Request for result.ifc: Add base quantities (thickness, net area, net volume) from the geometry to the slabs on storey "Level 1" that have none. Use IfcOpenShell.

First a look at what the model holds.

```python
import ifcopenshell
import ifcopenshell.util.element
import ifcopenshell.util.unit

model = ifcopenshell.open("result.ifc")
print(model.schema)
for unit_type in ("LENGTHUNIT", "AREAUNIT", "VOLUMEUNIT"):
    print(unit_type, ifcopenshell.util.unit.calculate_unit_scale(model, unit_type))
storey = next(s for s in model.by_type("IfcBuildingStorey") if s.Name == "Level 1")
slabs = [e for e in ifcopenshell.util.element.get_decomposition(storey) if e.is_a("IfcSlab")]
for e in sorted(slabs, key=lambda e: e.id()):
    print(e.id(), e.is_a(), e.Name, list(ifcopenshell.util.element.get_psets(e, qtos_only=True)), sep=" | ")
```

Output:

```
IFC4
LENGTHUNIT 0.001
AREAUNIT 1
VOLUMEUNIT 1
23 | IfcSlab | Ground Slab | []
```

```python
import ifcopenshell
import ifcopenshell.api.pset
import ifcopenshell.geom
import ifcopenshell.util.element
import ifcopenshell.util.shape
import ifcopenshell.util.unit

model = ifcopenshell.open("result.ifc")
unit_scale = ifcopenshell.util.unit.calculate_unit_scale(model)
area_scale = ifcopenshell.util.unit.calculate_unit_scale(model, "AREAUNIT")
volume_scale = ifcopenshell.util.unit.calculate_unit_scale(model, "VOLUMEUNIT")
settings = ifcopenshell.geom.settings()

storey = next(s for s in model.by_type("IfcBuildingStorey") if s.Name == "Level 1")
slabs = [e for e in ifcopenshell.util.element.get_decomposition(storey) if e.is_a("IfcSlab")]

for e in sorted(slabs, key=lambda e: e.id()):
    if ifcopenshell.util.element.get_psets(e, qtos_only=True, should_inherit=False):
        continue
    # Geometry comes back in metres, in the element's own axes.
    shape = ifcopenshell.geom.create_shape(settings, e)
    values = {
        "Width": ifcopenshell.util.shape.get_z(shape.geometry) / unit_scale,
        "NetArea": ifcopenshell.util.shape.get_footprint_area(shape.geometry) / area_scale,
        "NetVolume": ifcopenshell.util.shape.get_volume(shape.geometry) / volume_scale,
    }
    qto = ifcopenshell.api.pset.add_qto(model, product=e, name="Qto_SlabBaseQuantities")
    ifcopenshell.api.pset.edit_qto(model, qto=qto, properties=values)
    print(e.id(), {k: round(v, 3) for k, v in values.items()})

model.write("result_v2.ifc")
```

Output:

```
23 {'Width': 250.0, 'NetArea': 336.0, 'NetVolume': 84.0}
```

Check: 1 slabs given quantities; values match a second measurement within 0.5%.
